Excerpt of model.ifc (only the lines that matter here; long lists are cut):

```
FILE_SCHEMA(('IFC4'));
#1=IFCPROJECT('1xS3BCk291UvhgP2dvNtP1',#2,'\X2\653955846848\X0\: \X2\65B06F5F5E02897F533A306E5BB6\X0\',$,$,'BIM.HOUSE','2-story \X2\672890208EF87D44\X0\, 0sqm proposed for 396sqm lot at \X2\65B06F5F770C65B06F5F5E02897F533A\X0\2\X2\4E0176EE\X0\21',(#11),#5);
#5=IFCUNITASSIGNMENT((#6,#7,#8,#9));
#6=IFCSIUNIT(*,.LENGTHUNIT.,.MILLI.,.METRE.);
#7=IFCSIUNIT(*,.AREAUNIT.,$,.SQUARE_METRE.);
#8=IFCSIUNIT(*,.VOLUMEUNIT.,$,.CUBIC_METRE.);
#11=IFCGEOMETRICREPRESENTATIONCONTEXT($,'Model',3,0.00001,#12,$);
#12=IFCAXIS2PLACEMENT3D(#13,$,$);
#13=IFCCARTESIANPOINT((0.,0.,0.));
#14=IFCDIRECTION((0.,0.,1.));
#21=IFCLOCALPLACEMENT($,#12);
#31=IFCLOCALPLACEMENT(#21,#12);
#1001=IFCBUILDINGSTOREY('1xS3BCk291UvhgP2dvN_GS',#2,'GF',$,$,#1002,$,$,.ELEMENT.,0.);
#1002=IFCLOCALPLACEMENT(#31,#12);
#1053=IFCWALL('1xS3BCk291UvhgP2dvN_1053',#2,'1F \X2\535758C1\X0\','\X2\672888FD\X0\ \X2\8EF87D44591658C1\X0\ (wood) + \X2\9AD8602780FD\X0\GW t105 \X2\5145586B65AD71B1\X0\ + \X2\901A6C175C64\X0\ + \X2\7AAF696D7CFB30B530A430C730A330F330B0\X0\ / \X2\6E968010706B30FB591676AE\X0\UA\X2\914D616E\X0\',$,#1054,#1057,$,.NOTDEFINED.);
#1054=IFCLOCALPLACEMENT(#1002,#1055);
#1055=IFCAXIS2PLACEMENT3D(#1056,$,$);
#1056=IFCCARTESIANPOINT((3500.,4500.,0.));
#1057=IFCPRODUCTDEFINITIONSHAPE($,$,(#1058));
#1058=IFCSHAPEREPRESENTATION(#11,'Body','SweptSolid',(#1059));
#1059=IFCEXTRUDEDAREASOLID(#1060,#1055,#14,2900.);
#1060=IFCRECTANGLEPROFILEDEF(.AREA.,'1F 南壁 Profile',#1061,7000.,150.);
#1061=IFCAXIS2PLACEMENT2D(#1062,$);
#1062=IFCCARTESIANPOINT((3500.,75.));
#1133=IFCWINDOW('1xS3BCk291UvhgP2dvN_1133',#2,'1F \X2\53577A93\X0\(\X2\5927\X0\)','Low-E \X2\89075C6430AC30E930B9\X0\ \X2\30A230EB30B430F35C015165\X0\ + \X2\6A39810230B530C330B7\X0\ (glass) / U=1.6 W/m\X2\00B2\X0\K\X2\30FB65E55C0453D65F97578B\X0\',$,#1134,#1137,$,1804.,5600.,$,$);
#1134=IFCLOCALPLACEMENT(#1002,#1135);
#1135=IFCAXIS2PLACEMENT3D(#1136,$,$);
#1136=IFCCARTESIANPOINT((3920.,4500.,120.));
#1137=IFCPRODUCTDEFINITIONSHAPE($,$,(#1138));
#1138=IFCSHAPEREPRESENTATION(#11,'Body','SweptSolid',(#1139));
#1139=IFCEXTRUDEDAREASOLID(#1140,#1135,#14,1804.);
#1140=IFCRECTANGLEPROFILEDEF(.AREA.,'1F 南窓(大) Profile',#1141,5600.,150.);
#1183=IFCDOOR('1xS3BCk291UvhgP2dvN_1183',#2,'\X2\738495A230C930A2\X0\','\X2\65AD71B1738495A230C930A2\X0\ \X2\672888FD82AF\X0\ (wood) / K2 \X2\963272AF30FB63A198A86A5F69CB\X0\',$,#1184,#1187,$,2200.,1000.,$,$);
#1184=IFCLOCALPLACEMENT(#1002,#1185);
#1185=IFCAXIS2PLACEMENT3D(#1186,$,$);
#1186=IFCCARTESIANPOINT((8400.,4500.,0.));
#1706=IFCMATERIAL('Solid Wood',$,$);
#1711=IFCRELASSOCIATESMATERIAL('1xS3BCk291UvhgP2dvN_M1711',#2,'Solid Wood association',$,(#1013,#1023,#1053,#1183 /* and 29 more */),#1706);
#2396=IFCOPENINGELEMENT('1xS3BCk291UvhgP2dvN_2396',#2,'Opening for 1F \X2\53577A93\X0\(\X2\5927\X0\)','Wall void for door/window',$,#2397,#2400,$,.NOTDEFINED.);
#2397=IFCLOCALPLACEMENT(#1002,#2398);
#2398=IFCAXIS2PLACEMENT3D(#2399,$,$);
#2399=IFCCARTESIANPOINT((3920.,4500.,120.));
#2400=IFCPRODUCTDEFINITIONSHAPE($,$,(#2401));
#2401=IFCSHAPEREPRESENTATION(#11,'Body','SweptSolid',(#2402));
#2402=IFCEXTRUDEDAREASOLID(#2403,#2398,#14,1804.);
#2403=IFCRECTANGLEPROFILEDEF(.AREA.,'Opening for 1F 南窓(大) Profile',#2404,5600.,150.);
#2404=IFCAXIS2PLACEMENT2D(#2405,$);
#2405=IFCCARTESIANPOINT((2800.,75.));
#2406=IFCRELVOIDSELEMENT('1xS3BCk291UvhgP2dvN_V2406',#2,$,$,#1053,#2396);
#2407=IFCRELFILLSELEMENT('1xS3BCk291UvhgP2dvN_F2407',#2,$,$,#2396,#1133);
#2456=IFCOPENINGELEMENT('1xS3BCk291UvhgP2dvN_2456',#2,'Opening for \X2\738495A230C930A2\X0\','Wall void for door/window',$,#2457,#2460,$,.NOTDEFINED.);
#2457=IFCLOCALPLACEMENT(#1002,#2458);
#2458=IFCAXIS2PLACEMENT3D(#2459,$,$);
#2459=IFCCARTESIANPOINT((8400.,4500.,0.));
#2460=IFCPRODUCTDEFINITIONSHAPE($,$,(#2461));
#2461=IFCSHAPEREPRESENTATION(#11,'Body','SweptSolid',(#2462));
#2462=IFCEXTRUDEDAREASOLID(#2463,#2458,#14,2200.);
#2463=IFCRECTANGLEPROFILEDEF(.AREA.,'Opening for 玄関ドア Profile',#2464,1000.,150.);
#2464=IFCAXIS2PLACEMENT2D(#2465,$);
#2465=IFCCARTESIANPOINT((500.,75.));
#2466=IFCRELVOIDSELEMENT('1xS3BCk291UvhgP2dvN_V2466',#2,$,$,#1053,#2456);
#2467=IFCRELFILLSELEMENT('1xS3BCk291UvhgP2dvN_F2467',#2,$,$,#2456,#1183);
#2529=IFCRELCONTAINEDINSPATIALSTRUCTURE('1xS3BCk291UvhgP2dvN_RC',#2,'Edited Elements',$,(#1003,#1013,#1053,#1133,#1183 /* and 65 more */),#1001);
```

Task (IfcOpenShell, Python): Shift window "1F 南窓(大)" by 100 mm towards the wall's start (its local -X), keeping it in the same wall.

```python
import ifcopenshell
import ifcopenshell.api.geometry
import ifcopenshell.util.placement
import ifcopenshell.util.unit

model = ifcopenshell.open("model.ifc")
unit_scale = ifcopenshell.util.unit.calculate_unit_scale(model)

window = model.by_guid("1xS3BCk291UvhgP2dvN_1133")
opening = window.FillsVoids[0].RelatingOpeningElement
wall = opening.VoidsElements[0].RelatingBuildingElement

wall_matrix = ifcopenshell.util.placement.get_local_placement(wall.ObjectPlacement)
shift = wall_matrix[:3, 0] * -0.1 / unit_scale
before = ifcopenshell.util.placement.get_local_placement(window.ObjectPlacement)[:3, 3].copy()

# The window is not placed relative to its opening, so move both.
for product in (opening, window):
    matrix = ifcopenshell.util.placement.get_local_placement(product.ObjectPlacement)
    matrix[:3, 3] += shift
    ifcopenshell.api.geometry.edit_object_placement(model, product=product, matrix=matrix, is_si=False)

after = ifcopenshell.util.placement.get_local_placement(window.ObjectPlacement)[:3, 3]
print("window moved by", (after - before).round(3) + 0.0)

model.write("model_edited.ifc")
```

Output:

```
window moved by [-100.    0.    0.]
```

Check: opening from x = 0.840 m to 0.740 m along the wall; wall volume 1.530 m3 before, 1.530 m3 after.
